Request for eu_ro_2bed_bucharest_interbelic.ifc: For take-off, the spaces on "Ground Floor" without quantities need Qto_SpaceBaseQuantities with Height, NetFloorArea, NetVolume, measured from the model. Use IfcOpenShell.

First a look at what the model holds.

```python
import ifcopenshell
import ifcopenshell.util.element
import ifcopenshell.util.unit

model = ifcopenshell.open("eu_ro_2bed_bucharest_interbelic.ifc")
print(model.schema)
for unit_type in ("LENGTHUNIT", "AREAUNIT", "VOLUMEUNIT"):
    print(unit_type, ifcopenshell.util.unit.calculate_unit_scale(model, unit_type))
storey = next(s for s in model.by_type("IfcBuildingStorey") if s.Name == "Ground Floor")
spaces = [e for e in ifcopenshell.util.element.get_decomposition(storey) if e.is_a("IfcSpace")]
for e in sorted(spaces, key=lambda e: e.id()):
    print(e.id(), e.is_a(), e.Name, list(ifcopenshell.util.element.get_psets(e, qtos_only=True)), sep=" | ")
```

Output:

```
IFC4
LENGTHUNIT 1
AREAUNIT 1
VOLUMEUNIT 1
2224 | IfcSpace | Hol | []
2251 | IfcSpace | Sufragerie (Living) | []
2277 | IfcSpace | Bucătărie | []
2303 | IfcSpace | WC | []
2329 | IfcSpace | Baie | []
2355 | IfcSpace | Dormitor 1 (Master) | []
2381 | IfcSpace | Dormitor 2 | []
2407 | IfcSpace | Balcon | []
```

```python
import ifcopenshell
import ifcopenshell.api.pset
import ifcopenshell.geom
import ifcopenshell.util.element
import ifcopenshell.util.shape
import ifcopenshell.util.unit

model = ifcopenshell.open("eu_ro_2bed_bucharest_interbelic.ifc")
unit_scale = ifcopenshell.util.unit.calculate_unit_scale(model)
area_scale = ifcopenshell.util.unit.calculate_unit_scale(model, "AREAUNIT")
volume_scale = ifcopenshell.util.unit.calculate_unit_scale(model, "VOLUMEUNIT")
settings = ifcopenshell.geom.settings()

storey = next(s for s in model.by_type("IfcBuildingStorey") if s.Name == "Ground Floor")
spaces = [e for e in ifcopenshell.util.element.get_decomposition(storey) if e.is_a("IfcSpace")]

for e in sorted(spaces, key=lambda e: e.id()):
    if ifcopenshell.util.element.get_psets(e, qtos_only=True, should_inherit=False):
        continue
    # Geometry comes back in metres, in the element's own axes.
    shape = ifcopenshell.geom.create_shape(settings, e)
    values = {
        "Height": ifcopenshell.util.shape.get_z(shape.geometry) / unit_scale,
        "NetFloorArea": ifcopenshell.util.shape.get_footprint_area(shape.geometry) / area_scale,
        "NetVolume": ifcopenshell.util.shape.get_volume(shape.geometry) / volume_scale,
    }
    qto = ifcopenshell.api.pset.add_qto(model, product=e, name="Qto_SpaceBaseQuantities")
    ifcopenshell.api.pset.edit_qto(model, qto=qto, properties=values)
    print(e.id(), {k: round(v, 3) for k, v in values.items()})

model.write("eu_ro_2bed_bucharest_interbelic_updated.ifc")
```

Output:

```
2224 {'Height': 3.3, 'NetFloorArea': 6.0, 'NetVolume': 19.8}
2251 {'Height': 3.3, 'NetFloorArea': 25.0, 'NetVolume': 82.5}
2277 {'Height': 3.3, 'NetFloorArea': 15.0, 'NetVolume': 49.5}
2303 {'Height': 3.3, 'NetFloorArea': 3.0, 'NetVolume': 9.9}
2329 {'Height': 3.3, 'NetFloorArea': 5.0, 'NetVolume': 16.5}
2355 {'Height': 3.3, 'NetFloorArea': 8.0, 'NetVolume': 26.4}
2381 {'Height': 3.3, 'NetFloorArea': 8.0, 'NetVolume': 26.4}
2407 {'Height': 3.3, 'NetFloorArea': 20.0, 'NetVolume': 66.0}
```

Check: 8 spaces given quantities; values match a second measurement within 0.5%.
